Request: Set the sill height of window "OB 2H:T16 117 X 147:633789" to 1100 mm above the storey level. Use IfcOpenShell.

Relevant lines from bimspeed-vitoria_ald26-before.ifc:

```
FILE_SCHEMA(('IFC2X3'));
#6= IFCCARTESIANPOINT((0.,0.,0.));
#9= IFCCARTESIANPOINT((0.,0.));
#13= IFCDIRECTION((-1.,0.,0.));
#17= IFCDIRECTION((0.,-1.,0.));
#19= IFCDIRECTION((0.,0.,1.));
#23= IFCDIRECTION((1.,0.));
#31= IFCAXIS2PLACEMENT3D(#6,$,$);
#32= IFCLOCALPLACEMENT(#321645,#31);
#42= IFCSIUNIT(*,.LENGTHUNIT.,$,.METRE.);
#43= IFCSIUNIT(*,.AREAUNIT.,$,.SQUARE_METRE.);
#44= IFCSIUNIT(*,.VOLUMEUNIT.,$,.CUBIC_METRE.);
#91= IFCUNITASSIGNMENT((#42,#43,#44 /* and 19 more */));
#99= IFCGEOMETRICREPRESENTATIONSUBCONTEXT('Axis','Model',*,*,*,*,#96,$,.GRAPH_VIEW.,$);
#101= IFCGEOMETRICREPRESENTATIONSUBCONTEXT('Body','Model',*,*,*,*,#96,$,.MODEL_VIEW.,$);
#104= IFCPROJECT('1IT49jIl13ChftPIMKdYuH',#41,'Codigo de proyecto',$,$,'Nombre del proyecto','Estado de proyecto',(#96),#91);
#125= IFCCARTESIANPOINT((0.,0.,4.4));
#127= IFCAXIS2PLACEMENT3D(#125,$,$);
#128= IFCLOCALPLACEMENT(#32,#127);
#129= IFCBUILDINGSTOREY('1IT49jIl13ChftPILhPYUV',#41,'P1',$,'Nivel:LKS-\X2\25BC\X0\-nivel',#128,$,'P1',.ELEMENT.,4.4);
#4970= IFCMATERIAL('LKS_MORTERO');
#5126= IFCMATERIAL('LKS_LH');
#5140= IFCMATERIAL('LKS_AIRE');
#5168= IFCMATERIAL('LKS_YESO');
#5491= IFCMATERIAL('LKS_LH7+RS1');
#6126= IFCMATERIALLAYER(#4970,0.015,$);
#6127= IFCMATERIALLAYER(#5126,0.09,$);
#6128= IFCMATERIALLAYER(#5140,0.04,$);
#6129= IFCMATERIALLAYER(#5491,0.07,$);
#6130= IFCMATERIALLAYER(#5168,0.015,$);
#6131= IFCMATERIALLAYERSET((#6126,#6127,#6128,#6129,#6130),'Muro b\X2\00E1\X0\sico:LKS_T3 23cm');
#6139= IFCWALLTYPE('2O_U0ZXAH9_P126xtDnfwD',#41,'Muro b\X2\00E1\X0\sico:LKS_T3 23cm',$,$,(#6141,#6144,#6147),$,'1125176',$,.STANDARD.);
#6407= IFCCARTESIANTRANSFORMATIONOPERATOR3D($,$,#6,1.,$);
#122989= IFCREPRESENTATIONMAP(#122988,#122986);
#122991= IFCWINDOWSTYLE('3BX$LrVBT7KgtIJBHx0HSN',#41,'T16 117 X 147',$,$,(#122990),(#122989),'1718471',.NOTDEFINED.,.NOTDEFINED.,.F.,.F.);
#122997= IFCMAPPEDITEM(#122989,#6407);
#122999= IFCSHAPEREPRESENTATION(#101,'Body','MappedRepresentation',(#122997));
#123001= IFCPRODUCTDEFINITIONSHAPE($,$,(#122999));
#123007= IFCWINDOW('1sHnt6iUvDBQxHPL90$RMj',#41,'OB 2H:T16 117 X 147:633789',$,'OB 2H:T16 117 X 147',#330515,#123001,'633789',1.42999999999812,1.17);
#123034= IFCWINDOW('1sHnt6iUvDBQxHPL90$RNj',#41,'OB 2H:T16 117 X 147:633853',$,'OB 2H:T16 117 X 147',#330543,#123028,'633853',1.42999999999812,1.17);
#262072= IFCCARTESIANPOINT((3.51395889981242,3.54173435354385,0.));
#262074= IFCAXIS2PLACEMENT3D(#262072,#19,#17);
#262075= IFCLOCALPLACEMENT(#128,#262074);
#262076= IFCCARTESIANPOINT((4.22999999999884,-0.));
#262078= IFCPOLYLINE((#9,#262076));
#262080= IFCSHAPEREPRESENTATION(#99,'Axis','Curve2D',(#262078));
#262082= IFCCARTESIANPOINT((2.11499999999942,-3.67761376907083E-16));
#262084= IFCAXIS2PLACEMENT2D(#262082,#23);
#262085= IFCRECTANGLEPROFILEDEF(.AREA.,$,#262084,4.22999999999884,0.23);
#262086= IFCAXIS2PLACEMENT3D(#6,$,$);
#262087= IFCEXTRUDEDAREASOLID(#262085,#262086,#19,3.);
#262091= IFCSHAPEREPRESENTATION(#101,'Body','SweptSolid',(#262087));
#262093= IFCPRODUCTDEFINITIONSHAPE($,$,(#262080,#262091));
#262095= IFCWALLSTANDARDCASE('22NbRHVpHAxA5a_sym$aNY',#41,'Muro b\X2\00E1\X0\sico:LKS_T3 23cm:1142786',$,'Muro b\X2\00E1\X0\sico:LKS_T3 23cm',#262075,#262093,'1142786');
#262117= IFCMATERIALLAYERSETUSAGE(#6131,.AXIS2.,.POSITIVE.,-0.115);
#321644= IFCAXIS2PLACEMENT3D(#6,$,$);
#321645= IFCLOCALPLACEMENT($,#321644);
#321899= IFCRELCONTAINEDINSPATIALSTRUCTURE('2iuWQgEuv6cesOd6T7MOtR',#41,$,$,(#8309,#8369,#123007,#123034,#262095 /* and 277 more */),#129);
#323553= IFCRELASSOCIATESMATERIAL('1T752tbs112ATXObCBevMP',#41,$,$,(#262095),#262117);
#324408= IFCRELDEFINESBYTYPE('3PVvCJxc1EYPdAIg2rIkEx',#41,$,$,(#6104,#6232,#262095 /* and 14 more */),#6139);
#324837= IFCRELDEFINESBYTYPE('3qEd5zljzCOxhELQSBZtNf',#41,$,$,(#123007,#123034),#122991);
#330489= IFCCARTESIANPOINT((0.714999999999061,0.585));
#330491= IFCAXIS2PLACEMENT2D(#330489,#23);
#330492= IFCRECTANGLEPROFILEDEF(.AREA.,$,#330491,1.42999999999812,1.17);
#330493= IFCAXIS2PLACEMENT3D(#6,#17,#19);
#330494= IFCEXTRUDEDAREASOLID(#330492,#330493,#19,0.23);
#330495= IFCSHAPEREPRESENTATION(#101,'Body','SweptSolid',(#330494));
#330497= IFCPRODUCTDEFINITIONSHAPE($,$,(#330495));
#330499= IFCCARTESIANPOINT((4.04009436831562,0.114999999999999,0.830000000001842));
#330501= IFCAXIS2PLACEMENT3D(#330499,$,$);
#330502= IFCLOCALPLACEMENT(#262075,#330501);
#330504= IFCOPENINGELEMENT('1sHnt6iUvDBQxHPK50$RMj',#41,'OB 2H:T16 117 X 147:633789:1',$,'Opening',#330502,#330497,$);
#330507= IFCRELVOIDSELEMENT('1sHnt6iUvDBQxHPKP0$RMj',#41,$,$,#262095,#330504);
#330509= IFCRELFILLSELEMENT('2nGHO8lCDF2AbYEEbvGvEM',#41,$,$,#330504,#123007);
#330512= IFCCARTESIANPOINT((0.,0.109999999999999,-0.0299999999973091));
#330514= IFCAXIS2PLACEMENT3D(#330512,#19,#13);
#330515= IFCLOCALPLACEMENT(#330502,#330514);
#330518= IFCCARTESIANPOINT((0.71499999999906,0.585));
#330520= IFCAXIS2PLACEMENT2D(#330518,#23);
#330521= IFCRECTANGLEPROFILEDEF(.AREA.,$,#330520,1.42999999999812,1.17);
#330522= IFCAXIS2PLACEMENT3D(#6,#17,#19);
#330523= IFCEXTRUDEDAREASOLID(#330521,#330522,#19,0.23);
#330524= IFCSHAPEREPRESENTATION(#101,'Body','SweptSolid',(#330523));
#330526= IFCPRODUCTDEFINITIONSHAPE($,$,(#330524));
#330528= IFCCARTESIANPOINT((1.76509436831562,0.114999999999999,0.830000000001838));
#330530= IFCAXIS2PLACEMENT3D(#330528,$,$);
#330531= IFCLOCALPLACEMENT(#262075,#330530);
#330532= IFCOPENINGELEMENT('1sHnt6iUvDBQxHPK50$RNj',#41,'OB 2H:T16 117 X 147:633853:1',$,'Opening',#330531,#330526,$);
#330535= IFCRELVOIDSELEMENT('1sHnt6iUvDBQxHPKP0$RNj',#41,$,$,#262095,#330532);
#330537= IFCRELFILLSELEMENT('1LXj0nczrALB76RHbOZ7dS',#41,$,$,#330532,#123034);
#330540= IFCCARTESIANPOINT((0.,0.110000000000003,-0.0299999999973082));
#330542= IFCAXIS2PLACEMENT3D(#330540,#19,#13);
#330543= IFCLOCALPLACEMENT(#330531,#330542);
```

```python
import numpy as np
import ifcopenshell
import ifcopenshell.api.geometry
import ifcopenshell.geom
import ifcopenshell.util.element
import ifcopenshell.util.placement
import ifcopenshell.util.shape
import ifcopenshell.util.unit

model = ifcopenshell.open("bimspeed-vitoria_ald26-before.ifc")
unit_scale = ifcopenshell.util.unit.calculate_unit_scale(model)

window = model.by_guid("1sHnt6iUvDBQxHPL90$RMj")
opening = window.FillsVoids[0].RelatingOpeningElement
storey = ifcopenshell.util.element.get_container(window, ifc_class="IfcBuildingStorey")
level = ifcopenshell.util.placement.get_local_placement(storey.ObjectPlacement)[2, 3]

# The opening's origin need not be at the sill, so measure its lowest point.
shape = ifcopenshell.geom.create_shape(ifcopenshell.geom.settings(), opening)
bottom = ifcopenshell.util.shape.get_shape_bottom_elevation(shape, shape.geometry) / unit_scale
dz = level + 1.1 - bottom

shift = np.array([0.0, 0.0, dz])
# The window is placed relative to its opening, so it follows when the opening moves.
matrix = ifcopenshell.util.placement.get_local_placement(opening.ObjectPlacement)
matrix[:3, 3] += shift
ifcopenshell.api.geometry.edit_object_placement(
    model, product=opening, matrix=matrix, is_si=False, should_transform_children=True
)

print(f"moved by {dz * unit_scale:+.3f} m")

model.write("bimspeed-vitoria_ald26-before-out.ifc")
```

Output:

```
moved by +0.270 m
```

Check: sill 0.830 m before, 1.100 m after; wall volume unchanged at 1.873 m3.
